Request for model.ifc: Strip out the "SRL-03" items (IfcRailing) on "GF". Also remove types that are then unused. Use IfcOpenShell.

First a look at what the model holds.

```python
import ifcopenshell
import ifcopenshell.util.element

model = ifcopenshell.open("model.ifc")
print(model.schema)
storey = next(s for s in model.by_type("IfcBuildingStorey") if s.Name == "GF")
railings = [e for e in ifcopenshell.util.element.get_decomposition(storey) if e.is_a("IfcRailing")]
seen = {}
for e in railings:
    element_type = ifcopenshell.util.element.get_type(e)
    name = element_type.Name if element_type not in (None, e) else None
    seen[name] = seen.get(name, 0) + 1
for name, count in sorted(seen.items(), key=str):
    print(count, "x", name)
```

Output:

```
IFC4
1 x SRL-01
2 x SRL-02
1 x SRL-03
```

```python
import ifcopenshell
import ifcopenshell.api.root
import ifcopenshell.util.element

model = ifcopenshell.open("model.ifc")

storey = next(s for s in model.by_type("IfcBuildingStorey") if s.Name == "GF")
railings = [e for e in ifcopenshell.util.element.get_decomposition(storey) if e.is_a("IfcRailing")]
targets = [e for e in railings if (t := ifcopenshell.util.element.get_type(e)) not in (None, e) and t.Name == "SRL-03"]
types = {ifcopenshell.util.element.get_type(e) for e in targets} - {None, *targets}

for e in targets:
    ifcopenshell.api.root.remove_product(model, product=e)
print(len(targets), "removed")

unused = [t for t in types if not ifcopenshell.util.element.get_types(t)]
for t in unused:
    ifcopenshell.api.root.remove_product(model, product=t)
print(len(unused), "unused types removed")

model.write("model-out.ifc")
```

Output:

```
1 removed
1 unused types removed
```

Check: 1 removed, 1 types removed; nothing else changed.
